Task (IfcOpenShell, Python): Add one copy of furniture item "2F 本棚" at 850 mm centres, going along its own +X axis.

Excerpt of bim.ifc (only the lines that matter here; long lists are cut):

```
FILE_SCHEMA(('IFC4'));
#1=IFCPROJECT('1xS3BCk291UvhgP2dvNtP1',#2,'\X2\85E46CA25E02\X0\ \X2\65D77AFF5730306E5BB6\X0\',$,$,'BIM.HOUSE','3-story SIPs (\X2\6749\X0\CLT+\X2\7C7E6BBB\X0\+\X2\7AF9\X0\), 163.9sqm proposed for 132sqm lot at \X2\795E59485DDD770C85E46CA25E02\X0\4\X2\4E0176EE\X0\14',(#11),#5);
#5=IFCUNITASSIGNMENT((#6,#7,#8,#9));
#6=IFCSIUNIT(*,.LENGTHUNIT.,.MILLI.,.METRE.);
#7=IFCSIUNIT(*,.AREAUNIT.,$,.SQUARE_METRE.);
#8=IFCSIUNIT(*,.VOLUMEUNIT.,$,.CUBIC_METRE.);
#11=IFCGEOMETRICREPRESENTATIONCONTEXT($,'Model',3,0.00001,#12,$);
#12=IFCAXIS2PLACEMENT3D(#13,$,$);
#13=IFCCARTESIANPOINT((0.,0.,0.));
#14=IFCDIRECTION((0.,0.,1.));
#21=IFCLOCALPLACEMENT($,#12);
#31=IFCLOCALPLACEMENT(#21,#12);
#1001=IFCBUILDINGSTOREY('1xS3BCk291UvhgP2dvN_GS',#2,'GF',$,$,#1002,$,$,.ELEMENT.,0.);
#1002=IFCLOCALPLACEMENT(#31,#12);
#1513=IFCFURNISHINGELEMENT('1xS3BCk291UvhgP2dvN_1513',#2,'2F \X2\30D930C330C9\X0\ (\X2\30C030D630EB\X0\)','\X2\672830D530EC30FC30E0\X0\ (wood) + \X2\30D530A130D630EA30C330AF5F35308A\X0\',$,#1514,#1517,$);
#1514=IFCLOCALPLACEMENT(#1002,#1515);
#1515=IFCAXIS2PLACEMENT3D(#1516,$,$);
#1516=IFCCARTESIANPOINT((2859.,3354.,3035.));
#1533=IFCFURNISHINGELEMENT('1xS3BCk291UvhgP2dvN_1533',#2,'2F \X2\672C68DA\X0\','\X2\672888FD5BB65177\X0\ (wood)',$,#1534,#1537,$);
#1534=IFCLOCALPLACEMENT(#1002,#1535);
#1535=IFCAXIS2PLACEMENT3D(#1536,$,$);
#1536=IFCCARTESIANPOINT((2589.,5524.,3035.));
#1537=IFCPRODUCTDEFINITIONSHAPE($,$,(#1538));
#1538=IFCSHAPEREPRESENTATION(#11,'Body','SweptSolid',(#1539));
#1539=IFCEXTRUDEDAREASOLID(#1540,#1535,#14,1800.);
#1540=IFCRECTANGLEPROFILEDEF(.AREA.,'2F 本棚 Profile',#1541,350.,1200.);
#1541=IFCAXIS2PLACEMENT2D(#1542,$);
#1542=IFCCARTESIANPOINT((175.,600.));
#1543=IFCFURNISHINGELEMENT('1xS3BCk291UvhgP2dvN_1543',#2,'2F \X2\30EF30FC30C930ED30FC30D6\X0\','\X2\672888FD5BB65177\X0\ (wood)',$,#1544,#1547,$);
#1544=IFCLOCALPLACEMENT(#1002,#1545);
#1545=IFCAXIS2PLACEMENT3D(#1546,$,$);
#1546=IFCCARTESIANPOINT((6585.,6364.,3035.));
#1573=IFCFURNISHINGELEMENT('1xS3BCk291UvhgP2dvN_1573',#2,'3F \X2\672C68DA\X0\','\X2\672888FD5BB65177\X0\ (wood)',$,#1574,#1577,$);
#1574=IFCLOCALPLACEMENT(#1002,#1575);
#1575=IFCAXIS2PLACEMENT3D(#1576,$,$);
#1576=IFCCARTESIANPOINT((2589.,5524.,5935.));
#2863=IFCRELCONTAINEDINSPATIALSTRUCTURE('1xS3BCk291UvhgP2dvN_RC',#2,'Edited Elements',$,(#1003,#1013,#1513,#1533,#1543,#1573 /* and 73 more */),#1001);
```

```python
import ifcopenshell
import ifcopenshell.api.geometry
import ifcopenshell.api.root
import ifcopenshell.util.element
import ifcopenshell.util.placement

model = ifcopenshell.open("bim.ifc")


def reuse_history(source, copy):
    """copy_class also copies each property set's owner history, people and application; keep the originals."""
    for rel in copy.IsDefinedBy:
        if rel.is_a("IfcRelDefinesByProperties") and (history := rel.RelatingPropertyDefinition.OwnerHistory):
            rel.RelatingPropertyDefinition.OwnerHistory = source.OwnerHistory
            ifcopenshell.util.element.remove_deep2(model, history)


source = model.by_guid("1xS3BCk291UvhgP2dvN_1533")
base = ifcopenshell.util.placement.get_local_placement(source.ObjectPlacement)
step = base[:3, 0] * 850.0

for i in range(1, 2):
    copy = ifcopenshell.api.root.copy_class(model, product=source)
    copy.Representation = ifcopenshell.util.element.copy_deep(
        model, source.Representation, exclude=["IfcGeometricRepresentationContext", "IfcRepresentationMap"]
    )
    reuse_history(source, copy)
    matrix = base.copy()
    matrix[:3, 3] += i * step
    print("added at", matrix[:3, 3].round(3) + 0.0)
    ifcopenshell.api.geometry.edit_object_placement(model, product=copy, matrix=matrix, is_si=False)

model.write("bim_v2.ifc")
```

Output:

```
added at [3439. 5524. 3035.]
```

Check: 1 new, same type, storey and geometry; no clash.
